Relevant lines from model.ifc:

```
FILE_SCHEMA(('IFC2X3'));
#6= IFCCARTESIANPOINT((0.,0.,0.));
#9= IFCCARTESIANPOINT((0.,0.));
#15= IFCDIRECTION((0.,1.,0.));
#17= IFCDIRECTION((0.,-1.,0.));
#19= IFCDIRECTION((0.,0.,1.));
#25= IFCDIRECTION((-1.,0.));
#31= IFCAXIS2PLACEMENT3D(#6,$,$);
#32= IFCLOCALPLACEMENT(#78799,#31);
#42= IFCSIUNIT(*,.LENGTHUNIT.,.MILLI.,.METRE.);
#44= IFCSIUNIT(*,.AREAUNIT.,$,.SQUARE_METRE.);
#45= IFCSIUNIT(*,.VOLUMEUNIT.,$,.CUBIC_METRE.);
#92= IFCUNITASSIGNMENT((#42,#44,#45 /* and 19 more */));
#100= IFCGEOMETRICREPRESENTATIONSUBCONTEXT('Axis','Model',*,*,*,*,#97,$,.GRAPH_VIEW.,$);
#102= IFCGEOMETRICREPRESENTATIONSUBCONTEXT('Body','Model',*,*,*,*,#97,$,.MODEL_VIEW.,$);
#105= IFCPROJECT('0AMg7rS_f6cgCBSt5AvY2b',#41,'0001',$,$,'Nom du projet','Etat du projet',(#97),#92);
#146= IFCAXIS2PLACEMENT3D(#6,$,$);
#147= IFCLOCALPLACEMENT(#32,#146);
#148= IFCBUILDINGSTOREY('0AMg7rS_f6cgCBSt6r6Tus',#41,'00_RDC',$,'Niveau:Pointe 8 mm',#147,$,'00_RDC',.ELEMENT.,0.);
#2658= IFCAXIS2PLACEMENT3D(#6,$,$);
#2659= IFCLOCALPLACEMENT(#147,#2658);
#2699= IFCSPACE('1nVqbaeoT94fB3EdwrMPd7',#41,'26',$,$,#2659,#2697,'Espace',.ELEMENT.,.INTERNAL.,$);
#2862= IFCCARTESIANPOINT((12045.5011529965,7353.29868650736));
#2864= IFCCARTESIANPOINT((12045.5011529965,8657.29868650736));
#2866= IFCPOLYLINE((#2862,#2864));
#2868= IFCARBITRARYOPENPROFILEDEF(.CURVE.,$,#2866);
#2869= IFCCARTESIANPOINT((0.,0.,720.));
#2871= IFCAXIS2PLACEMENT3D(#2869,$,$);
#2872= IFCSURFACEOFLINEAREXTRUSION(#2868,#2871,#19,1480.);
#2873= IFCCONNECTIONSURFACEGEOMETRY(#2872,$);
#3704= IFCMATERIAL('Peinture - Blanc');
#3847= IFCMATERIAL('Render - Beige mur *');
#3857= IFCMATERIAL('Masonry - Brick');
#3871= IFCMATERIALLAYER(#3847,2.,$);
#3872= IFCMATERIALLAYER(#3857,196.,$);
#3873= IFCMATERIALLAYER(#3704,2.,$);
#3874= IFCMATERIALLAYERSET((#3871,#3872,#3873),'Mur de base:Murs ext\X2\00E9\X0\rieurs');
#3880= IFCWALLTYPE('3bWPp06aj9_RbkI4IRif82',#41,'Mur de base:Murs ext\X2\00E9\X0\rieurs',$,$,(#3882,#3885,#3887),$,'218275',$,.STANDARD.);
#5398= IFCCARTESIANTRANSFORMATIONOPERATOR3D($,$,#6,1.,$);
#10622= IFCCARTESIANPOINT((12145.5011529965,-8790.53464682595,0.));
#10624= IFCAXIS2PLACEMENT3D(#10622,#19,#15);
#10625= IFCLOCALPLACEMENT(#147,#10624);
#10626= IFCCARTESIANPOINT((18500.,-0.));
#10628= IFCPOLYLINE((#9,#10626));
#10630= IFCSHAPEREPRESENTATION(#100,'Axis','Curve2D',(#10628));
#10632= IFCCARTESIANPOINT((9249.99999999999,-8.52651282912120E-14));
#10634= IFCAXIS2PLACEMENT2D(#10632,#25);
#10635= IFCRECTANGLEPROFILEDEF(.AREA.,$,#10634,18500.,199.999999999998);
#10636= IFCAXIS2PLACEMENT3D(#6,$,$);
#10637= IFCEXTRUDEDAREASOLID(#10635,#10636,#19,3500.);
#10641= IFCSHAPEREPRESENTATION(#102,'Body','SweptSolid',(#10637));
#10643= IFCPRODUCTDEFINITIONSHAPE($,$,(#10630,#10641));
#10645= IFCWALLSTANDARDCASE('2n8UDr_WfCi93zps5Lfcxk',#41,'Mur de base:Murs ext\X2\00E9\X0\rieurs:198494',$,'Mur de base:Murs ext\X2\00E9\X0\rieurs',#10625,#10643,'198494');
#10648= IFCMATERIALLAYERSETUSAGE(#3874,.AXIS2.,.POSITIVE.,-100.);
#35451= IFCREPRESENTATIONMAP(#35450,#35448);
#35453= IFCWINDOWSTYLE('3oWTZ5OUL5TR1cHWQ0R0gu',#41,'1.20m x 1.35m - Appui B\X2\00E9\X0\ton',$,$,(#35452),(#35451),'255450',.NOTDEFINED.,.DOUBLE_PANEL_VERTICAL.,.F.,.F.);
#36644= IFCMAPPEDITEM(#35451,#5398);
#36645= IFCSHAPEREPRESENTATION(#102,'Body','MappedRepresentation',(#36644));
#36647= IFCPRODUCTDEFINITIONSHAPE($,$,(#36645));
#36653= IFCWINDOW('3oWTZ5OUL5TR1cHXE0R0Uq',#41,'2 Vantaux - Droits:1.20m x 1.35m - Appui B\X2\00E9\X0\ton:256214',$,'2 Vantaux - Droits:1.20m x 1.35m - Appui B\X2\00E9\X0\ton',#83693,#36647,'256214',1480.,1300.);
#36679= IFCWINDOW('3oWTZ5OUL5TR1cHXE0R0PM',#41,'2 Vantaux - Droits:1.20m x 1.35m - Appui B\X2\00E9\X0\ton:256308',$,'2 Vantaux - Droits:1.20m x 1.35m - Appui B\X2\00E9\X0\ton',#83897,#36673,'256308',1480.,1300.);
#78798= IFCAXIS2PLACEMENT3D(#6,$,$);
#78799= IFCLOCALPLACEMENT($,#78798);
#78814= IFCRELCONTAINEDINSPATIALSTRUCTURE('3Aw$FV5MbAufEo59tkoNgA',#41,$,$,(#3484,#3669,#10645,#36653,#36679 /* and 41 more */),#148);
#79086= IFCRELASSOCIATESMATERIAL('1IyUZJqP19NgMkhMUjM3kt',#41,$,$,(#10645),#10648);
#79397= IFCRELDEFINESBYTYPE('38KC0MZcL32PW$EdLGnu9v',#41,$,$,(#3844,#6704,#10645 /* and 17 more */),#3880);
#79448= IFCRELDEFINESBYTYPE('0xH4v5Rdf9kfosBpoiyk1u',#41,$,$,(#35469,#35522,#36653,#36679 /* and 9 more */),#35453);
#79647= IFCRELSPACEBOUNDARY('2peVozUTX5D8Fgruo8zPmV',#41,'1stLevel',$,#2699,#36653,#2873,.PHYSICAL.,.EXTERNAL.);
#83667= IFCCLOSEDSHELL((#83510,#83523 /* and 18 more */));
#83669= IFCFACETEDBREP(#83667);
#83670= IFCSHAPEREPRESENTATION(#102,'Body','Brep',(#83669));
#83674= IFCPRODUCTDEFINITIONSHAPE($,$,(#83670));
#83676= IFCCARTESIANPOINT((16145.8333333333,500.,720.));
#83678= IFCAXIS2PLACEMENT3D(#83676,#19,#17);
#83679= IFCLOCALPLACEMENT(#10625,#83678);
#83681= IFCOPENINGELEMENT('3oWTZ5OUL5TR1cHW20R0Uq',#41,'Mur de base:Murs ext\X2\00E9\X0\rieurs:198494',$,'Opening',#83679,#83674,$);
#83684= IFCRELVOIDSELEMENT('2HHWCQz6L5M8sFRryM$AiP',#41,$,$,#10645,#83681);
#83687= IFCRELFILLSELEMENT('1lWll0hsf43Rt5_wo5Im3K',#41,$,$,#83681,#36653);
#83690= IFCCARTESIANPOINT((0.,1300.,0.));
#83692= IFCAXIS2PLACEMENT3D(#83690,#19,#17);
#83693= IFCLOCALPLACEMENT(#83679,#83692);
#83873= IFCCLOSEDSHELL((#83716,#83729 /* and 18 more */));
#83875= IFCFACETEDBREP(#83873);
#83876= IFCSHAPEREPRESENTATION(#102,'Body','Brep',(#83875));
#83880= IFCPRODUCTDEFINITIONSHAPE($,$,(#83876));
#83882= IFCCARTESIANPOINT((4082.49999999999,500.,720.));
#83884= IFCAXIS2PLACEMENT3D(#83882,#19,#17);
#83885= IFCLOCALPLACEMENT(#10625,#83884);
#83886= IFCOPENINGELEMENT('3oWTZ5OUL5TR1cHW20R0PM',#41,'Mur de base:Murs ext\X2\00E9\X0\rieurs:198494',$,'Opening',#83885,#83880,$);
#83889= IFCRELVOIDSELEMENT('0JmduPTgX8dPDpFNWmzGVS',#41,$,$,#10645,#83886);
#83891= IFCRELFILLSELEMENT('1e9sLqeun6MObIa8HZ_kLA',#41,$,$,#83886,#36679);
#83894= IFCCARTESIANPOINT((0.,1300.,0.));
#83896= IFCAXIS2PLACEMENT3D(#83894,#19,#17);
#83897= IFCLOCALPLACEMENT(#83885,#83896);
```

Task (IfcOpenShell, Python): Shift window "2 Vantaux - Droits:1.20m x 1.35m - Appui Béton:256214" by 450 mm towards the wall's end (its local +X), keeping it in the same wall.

```python
import numpy as np
import ifcopenshell
import ifcopenshell.api.geometry
import ifcopenshell.util.placement
import ifcopenshell.util.unit

model = ifcopenshell.open("model.ifc")
unit_scale = ifcopenshell.util.unit.calculate_unit_scale(model)

window = model.by_guid("3oWTZ5OUL5TR1cHXE0R0Uq")
opening = window.FillsVoids[0].RelatingOpeningElement
wall = opening.VoidsElements[0].RelatingBuildingElement

wall_matrix = ifcopenshell.util.placement.get_local_placement(wall.ObjectPlacement)
shift = wall_matrix[:3, 0] * 0.45 / unit_scale
before = ifcopenshell.util.placement.get_local_placement(window.ObjectPlacement)[:3, 3].copy()

# The window is placed relative to its opening, so it follows when the opening moves.
matrix = ifcopenshell.util.placement.get_local_placement(opening.ObjectPlacement)
matrix[:3, 3] += shift
ifcopenshell.api.geometry.edit_object_placement(
    model, product=opening, matrix=matrix, is_si=False, should_transform_children=True
)

# Space boundary surfaces are stored in each space's coordinates; move them too.
for rel in window.ProvidesBoundaries:
    if not rel.ConnectionGeometry:
        continue
    surface = rel.ConnectionGeometry.SurfaceOnRelatingElement
    space_matrix = ifcopenshell.util.placement.get_local_placement(rel.RelatingSpace.ObjectPlacement)
    point = np.array(surface.Position.Location.Coordinates) + space_matrix[:3, :3].T @ shift
    surface.Position = model.createIfcAxis2Placement3D(
        model.createIfcCartesianPoint(point.tolist()), surface.Position.Axis, surface.Position.RefDirection
    )

after = ifcopenshell.util.placement.get_local_placement(window.ObjectPlacement)[:3, 3]
print("window moved by", (after - before).round(3) + 0.0)

model.write("model_rev.ifc")
```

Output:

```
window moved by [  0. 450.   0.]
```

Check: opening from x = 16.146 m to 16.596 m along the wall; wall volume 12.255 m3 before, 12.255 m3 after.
